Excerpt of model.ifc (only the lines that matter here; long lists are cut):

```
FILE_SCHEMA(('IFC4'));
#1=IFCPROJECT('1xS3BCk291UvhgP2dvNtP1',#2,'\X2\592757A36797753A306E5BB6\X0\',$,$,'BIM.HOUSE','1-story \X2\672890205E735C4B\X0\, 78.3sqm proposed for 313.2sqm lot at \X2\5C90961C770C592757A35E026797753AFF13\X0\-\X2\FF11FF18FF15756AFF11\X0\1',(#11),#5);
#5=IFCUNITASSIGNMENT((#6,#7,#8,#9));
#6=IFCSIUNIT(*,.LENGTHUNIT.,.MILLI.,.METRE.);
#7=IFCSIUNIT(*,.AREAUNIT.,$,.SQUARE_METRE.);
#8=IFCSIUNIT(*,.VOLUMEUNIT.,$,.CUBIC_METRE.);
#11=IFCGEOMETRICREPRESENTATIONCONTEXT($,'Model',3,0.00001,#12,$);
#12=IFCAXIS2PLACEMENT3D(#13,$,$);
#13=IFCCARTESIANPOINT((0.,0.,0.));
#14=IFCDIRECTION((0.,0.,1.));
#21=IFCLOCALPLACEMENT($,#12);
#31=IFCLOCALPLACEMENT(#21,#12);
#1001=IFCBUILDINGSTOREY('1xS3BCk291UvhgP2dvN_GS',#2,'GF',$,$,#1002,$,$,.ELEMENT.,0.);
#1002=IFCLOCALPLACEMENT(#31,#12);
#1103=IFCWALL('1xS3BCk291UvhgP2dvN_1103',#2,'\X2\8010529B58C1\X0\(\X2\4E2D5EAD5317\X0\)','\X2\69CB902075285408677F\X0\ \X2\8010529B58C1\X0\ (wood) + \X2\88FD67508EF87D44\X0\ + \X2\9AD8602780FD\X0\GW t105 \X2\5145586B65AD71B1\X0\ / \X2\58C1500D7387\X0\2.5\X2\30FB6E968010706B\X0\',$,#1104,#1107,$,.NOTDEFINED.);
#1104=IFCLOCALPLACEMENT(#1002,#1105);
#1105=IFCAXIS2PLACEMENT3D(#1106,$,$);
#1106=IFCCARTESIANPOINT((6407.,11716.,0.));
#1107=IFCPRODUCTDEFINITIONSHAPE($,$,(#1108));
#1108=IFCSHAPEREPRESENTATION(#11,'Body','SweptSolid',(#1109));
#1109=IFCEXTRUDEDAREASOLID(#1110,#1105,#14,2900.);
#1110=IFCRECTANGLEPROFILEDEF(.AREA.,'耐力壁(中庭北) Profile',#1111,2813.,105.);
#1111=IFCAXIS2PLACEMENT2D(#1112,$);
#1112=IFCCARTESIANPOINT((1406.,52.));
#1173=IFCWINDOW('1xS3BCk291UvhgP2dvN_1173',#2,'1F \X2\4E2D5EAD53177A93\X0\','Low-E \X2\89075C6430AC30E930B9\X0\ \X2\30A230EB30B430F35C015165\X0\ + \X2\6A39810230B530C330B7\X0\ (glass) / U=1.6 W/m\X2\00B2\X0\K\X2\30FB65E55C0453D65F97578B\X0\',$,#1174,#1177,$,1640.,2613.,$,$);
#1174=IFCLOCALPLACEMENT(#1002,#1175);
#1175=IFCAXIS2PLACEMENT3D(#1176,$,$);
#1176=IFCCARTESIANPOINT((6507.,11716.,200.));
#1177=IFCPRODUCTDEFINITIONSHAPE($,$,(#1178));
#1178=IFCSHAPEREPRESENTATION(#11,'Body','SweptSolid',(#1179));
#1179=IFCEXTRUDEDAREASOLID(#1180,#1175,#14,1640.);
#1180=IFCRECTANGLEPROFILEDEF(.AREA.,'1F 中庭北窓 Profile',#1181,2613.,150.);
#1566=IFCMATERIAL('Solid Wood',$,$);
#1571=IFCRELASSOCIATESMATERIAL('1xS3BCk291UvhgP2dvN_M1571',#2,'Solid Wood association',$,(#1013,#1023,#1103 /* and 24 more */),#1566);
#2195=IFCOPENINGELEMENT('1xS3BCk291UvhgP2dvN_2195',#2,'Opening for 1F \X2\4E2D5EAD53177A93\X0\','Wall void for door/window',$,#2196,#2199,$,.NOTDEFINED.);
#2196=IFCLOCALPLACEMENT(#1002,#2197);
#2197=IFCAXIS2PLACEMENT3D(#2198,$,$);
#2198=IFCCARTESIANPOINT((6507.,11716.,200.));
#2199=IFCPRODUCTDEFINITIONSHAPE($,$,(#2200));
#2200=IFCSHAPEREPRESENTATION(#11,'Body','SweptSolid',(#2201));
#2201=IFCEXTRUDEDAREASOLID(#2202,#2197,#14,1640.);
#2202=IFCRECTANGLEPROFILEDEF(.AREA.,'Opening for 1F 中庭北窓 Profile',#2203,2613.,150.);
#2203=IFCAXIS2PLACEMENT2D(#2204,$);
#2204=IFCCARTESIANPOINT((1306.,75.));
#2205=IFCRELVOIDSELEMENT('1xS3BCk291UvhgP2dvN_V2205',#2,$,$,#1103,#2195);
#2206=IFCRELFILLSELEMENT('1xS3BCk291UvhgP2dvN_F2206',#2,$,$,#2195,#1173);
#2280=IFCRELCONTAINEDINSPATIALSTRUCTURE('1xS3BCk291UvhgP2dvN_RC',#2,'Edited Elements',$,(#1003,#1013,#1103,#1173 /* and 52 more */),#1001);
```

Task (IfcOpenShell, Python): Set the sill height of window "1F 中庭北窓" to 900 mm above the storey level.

```python
import numpy as np
import ifcopenshell
import ifcopenshell.api.geometry
import ifcopenshell.geom
import ifcopenshell.util.element
import ifcopenshell.util.placement
import ifcopenshell.util.shape
import ifcopenshell.util.unit

model = ifcopenshell.open("model.ifc")
unit_scale = ifcopenshell.util.unit.calculate_unit_scale(model)

window = model.by_guid("1xS3BCk291UvhgP2dvN_1173")
opening = window.FillsVoids[0].RelatingOpeningElement
storey = ifcopenshell.util.element.get_container(window, ifc_class="IfcBuildingStorey")
level = ifcopenshell.util.placement.get_local_placement(storey.ObjectPlacement)[2, 3]

# The opening's origin need not be at the sill, so measure its lowest point.
shape = ifcopenshell.geom.create_shape(ifcopenshell.geom.settings(), opening)
bottom = ifcopenshell.util.shape.get_shape_bottom_elevation(shape, shape.geometry) / unit_scale
dz = level + 900.0 - bottom

shift = np.array([0.0, 0.0, dz])
# The window is not placed relative to its opening, so move both.
for product in (opening, window):
    matrix = ifcopenshell.util.placement.get_local_placement(product.ObjectPlacement)
    matrix[:3, 3] += shift
    ifcopenshell.api.geometry.edit_object_placement(model, product=product, matrix=matrix, is_si=False)

print(f"moved by {dz * unit_scale:+.3f} m")

model.write("model_updated.ifc")
```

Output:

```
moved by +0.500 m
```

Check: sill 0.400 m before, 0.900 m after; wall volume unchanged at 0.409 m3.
